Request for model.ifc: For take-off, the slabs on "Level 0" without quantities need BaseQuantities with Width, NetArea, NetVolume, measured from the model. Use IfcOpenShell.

First a look at what the model holds.

```python
import ifcopenshell
import ifcopenshell.util.element
import ifcopenshell.util.unit

model = ifcopenshell.open("model.ifc")
print(model.schema)
for unit_type in ("LENGTHUNIT", "AREAUNIT", "VOLUMEUNIT"):
    print(unit_type, ifcopenshell.util.unit.calculate_unit_scale(model, unit_type))
storey = next(s for s in model.by_type("IfcBuildingStorey") if s.Name == "Level 0")
slabs = [e for e in ifcopenshell.util.element.get_decomposition(storey) if e.is_a("IfcSlab")]
for e in sorted(slabs, key=lambda e: e.id()):
    print(e.id(), e.is_a(), e.Name, list(ifcopenshell.util.element.get_psets(e, qtos_only=True)), sep=" | ")
```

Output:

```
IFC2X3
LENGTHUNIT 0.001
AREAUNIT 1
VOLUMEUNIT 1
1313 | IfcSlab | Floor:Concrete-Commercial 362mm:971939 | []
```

```python
import ifcopenshell
import ifcopenshell.api.pset
import ifcopenshell.geom
import ifcopenshell.util.element
import ifcopenshell.util.shape
import ifcopenshell.util.unit

model = ifcopenshell.open("model.ifc")
unit_scale = ifcopenshell.util.unit.calculate_unit_scale(model)
area_scale = ifcopenshell.util.unit.calculate_unit_scale(model, "AREAUNIT")
volume_scale = ifcopenshell.util.unit.calculate_unit_scale(model, "VOLUMEUNIT")
settings = ifcopenshell.geom.settings()

storey = next(s for s in model.by_type("IfcBuildingStorey") if s.Name == "Level 0")
slabs = [e for e in ifcopenshell.util.element.get_decomposition(storey) if e.is_a("IfcSlab")]

for e in sorted(slabs, key=lambda e: e.id()):
    if ifcopenshell.util.element.get_psets(e, qtos_only=True, should_inherit=False):
        continue
    # Geometry comes back in metres, in the element's own axes.
    shape = ifcopenshell.geom.create_shape(settings, e)
    values = {
        "Width": ifcopenshell.util.shape.get_z(shape.geometry) / unit_scale,
        "NetArea": ifcopenshell.util.shape.get_footprint_area(shape.geometry) / area_scale,
        "NetVolume": ifcopenshell.util.shape.get_volume(shape.geometry) / volume_scale,
    }
    qto = ifcopenshell.api.pset.add_qto(model, product=e, name="BaseQuantities")
    ifcopenshell.api.pset.edit_qto(model, qto=qto, properties=values)
    print(e.id(), {k: round(v, 3) for k, v in values.items()})

model.write("model_updated.ifc")
```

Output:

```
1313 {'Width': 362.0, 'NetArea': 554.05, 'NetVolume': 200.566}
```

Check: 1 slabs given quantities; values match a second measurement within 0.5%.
